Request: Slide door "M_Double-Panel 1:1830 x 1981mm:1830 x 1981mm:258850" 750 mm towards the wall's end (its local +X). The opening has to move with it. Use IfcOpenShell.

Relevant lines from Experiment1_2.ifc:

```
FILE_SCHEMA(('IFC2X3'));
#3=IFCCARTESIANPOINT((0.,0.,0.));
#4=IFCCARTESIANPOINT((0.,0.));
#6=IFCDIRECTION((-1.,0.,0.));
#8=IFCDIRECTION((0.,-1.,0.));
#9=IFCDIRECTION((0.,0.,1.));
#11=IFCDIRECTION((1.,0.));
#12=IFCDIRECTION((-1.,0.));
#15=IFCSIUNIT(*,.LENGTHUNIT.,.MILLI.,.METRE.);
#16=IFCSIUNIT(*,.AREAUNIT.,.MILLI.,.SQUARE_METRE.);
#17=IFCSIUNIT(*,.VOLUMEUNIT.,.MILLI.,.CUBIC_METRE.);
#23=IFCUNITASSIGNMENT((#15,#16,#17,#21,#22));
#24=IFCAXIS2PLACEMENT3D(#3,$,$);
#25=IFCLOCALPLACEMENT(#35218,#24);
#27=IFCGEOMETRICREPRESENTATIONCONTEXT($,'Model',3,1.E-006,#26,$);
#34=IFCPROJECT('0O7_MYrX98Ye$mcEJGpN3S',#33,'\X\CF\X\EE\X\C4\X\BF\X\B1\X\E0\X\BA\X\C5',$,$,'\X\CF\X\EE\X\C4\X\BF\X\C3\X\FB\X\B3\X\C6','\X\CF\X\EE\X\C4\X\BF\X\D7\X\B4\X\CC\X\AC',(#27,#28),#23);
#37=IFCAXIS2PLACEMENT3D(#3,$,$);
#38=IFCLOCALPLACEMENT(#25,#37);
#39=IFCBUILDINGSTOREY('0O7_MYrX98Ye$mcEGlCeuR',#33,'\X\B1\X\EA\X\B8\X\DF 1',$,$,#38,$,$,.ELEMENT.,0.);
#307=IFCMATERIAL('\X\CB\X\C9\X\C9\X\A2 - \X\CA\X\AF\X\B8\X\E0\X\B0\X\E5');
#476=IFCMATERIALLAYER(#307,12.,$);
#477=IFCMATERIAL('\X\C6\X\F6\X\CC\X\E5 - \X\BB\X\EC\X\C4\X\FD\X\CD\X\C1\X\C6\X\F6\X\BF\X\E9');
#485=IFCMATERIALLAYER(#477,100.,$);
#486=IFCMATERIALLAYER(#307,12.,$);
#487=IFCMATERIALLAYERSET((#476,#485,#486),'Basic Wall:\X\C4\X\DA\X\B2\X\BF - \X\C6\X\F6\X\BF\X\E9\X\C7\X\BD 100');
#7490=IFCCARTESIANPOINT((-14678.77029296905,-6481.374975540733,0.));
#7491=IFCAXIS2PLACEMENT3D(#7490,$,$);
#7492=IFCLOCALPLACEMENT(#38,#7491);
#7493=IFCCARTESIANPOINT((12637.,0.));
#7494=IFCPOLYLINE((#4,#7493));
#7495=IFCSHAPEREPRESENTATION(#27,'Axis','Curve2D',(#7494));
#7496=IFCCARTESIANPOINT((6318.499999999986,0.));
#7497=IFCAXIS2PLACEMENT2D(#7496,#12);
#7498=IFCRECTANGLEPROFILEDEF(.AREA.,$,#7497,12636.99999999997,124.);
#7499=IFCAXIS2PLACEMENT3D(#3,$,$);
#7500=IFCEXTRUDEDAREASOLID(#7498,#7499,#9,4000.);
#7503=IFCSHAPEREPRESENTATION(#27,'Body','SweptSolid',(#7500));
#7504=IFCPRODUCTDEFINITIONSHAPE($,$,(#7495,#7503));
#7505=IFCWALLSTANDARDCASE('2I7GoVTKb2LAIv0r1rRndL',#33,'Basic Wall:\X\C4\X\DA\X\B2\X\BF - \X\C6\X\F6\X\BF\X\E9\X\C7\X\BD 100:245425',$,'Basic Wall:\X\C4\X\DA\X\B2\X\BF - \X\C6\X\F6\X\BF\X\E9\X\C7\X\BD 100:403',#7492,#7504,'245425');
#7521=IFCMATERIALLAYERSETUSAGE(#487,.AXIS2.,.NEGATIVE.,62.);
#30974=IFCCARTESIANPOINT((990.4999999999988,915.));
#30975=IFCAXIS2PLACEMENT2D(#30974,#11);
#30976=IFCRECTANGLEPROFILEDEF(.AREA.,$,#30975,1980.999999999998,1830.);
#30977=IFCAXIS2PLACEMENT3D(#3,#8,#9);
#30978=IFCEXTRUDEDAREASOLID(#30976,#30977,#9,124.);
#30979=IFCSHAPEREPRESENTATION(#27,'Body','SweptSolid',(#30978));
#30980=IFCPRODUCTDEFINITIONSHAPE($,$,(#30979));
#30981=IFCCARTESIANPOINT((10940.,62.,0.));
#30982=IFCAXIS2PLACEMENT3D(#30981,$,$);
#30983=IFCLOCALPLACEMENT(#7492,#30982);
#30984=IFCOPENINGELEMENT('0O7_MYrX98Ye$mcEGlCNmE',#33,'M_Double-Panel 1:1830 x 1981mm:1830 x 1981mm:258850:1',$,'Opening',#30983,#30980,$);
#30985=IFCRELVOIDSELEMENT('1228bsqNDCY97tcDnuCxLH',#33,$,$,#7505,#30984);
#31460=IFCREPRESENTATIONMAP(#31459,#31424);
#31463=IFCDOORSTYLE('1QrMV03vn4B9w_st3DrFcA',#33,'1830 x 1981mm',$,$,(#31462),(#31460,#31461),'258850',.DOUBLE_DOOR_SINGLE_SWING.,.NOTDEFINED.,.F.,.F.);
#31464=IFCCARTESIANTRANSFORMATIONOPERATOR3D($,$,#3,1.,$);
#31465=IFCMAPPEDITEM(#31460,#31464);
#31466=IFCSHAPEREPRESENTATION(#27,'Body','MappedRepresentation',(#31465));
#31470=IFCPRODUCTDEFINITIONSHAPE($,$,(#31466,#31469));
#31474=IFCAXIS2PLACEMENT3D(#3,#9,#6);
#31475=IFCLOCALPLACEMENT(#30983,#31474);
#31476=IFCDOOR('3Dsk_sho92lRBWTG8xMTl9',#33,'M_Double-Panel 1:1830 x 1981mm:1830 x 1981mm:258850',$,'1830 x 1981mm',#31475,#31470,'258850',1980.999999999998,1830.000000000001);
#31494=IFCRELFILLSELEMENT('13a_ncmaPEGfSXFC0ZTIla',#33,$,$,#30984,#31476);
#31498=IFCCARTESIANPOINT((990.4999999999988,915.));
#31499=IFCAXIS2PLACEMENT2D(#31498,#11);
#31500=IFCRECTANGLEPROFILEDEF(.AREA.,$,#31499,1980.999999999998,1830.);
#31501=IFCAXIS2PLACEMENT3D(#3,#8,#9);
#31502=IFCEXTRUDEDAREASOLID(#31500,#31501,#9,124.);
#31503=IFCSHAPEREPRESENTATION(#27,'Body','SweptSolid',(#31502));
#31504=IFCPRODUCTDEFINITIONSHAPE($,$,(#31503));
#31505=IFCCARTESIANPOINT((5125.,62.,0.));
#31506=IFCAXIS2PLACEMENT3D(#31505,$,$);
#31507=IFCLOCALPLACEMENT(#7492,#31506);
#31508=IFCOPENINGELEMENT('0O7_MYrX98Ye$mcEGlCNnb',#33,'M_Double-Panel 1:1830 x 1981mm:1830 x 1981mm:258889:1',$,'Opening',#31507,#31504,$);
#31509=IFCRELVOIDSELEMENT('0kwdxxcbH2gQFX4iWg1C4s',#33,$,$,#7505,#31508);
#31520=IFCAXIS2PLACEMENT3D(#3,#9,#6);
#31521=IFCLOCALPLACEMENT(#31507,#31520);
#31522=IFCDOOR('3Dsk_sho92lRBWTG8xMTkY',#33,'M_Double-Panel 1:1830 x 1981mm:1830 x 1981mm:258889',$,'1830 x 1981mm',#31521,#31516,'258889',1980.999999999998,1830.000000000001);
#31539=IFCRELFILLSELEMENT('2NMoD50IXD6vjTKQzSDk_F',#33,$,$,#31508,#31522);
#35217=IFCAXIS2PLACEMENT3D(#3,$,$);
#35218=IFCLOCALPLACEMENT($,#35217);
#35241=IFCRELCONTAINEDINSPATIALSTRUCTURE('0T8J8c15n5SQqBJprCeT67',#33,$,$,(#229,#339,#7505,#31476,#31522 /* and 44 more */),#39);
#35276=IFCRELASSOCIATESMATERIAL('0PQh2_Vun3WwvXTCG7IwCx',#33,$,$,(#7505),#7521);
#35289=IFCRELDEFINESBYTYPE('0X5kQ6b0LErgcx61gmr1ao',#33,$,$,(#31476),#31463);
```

```python
import ifcopenshell
import ifcopenshell.api.geometry
import ifcopenshell.util.placement
import ifcopenshell.util.unit

model = ifcopenshell.open("Experiment1_2.ifc")
unit_scale = ifcopenshell.util.unit.calculate_unit_scale(model)

door = model.by_guid("3Dsk_sho92lRBWTG8xMTl9")
opening = door.FillsVoids[0].RelatingOpeningElement
wall = opening.VoidsElements[0].RelatingBuildingElement

wall_matrix = ifcopenshell.util.placement.get_local_placement(wall.ObjectPlacement)
shift = wall_matrix[:3, 0] * 0.75 / unit_scale
before = ifcopenshell.util.placement.get_local_placement(door.ObjectPlacement)[:3, 3].copy()

# The door is placed relative to its opening, so it follows when the opening moves.
matrix = ifcopenshell.util.placement.get_local_placement(opening.ObjectPlacement)
matrix[:3, 3] += shift
ifcopenshell.api.geometry.edit_object_placement(
    model, product=opening, matrix=matrix, is_si=False, should_transform_children=True
)

after = ifcopenshell.util.placement.get_local_placement(door.ObjectPlacement)[:3, 3]
print("door moved by", (after - before).round(3) + 0.0)

model.write("Experiment1_2_v2.ifc")
```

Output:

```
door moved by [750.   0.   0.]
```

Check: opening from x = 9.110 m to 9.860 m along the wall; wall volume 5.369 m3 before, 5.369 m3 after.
